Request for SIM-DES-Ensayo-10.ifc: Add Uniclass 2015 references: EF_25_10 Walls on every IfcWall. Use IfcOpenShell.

First a look at what the model holds.

```python
import ifcopenshell

model = ifcopenshell.open("SIM-DES-Ensayo-10.ifc")
print(model.schema)
print("classifications:", [c.Name for c in model.by_type("IfcClassification")])
for ifc_class in ("IfcDoor", "IfcRoof", "IfcStair", "IfcWall", "IfcWindow"):
    print(ifc_class, len(model.by_type(ifc_class)))
```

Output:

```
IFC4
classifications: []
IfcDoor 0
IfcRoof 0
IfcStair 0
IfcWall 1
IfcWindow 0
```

```python
import ifcopenshell
import ifcopenshell.api.classification

model = ifcopenshell.open("SIM-DES-Ensayo-10.ifc")

system = ifcopenshell.api.classification.add_classification(model, classification="Uniclass 2015")

codes = {
    "IfcWall": ("EF_25_10", "Walls"),
}
for ifc_class, (code, name) in codes.items():
    products = model.by_type(ifc_class)
    ifcopenshell.api.classification.add_reference(
        model, products=products, classification=system, identification=code, name=name
    )
    print(code, len(products))

model.write("SIM-DES-Ensayo-10_edited.ifc")
```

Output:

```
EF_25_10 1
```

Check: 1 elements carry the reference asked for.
